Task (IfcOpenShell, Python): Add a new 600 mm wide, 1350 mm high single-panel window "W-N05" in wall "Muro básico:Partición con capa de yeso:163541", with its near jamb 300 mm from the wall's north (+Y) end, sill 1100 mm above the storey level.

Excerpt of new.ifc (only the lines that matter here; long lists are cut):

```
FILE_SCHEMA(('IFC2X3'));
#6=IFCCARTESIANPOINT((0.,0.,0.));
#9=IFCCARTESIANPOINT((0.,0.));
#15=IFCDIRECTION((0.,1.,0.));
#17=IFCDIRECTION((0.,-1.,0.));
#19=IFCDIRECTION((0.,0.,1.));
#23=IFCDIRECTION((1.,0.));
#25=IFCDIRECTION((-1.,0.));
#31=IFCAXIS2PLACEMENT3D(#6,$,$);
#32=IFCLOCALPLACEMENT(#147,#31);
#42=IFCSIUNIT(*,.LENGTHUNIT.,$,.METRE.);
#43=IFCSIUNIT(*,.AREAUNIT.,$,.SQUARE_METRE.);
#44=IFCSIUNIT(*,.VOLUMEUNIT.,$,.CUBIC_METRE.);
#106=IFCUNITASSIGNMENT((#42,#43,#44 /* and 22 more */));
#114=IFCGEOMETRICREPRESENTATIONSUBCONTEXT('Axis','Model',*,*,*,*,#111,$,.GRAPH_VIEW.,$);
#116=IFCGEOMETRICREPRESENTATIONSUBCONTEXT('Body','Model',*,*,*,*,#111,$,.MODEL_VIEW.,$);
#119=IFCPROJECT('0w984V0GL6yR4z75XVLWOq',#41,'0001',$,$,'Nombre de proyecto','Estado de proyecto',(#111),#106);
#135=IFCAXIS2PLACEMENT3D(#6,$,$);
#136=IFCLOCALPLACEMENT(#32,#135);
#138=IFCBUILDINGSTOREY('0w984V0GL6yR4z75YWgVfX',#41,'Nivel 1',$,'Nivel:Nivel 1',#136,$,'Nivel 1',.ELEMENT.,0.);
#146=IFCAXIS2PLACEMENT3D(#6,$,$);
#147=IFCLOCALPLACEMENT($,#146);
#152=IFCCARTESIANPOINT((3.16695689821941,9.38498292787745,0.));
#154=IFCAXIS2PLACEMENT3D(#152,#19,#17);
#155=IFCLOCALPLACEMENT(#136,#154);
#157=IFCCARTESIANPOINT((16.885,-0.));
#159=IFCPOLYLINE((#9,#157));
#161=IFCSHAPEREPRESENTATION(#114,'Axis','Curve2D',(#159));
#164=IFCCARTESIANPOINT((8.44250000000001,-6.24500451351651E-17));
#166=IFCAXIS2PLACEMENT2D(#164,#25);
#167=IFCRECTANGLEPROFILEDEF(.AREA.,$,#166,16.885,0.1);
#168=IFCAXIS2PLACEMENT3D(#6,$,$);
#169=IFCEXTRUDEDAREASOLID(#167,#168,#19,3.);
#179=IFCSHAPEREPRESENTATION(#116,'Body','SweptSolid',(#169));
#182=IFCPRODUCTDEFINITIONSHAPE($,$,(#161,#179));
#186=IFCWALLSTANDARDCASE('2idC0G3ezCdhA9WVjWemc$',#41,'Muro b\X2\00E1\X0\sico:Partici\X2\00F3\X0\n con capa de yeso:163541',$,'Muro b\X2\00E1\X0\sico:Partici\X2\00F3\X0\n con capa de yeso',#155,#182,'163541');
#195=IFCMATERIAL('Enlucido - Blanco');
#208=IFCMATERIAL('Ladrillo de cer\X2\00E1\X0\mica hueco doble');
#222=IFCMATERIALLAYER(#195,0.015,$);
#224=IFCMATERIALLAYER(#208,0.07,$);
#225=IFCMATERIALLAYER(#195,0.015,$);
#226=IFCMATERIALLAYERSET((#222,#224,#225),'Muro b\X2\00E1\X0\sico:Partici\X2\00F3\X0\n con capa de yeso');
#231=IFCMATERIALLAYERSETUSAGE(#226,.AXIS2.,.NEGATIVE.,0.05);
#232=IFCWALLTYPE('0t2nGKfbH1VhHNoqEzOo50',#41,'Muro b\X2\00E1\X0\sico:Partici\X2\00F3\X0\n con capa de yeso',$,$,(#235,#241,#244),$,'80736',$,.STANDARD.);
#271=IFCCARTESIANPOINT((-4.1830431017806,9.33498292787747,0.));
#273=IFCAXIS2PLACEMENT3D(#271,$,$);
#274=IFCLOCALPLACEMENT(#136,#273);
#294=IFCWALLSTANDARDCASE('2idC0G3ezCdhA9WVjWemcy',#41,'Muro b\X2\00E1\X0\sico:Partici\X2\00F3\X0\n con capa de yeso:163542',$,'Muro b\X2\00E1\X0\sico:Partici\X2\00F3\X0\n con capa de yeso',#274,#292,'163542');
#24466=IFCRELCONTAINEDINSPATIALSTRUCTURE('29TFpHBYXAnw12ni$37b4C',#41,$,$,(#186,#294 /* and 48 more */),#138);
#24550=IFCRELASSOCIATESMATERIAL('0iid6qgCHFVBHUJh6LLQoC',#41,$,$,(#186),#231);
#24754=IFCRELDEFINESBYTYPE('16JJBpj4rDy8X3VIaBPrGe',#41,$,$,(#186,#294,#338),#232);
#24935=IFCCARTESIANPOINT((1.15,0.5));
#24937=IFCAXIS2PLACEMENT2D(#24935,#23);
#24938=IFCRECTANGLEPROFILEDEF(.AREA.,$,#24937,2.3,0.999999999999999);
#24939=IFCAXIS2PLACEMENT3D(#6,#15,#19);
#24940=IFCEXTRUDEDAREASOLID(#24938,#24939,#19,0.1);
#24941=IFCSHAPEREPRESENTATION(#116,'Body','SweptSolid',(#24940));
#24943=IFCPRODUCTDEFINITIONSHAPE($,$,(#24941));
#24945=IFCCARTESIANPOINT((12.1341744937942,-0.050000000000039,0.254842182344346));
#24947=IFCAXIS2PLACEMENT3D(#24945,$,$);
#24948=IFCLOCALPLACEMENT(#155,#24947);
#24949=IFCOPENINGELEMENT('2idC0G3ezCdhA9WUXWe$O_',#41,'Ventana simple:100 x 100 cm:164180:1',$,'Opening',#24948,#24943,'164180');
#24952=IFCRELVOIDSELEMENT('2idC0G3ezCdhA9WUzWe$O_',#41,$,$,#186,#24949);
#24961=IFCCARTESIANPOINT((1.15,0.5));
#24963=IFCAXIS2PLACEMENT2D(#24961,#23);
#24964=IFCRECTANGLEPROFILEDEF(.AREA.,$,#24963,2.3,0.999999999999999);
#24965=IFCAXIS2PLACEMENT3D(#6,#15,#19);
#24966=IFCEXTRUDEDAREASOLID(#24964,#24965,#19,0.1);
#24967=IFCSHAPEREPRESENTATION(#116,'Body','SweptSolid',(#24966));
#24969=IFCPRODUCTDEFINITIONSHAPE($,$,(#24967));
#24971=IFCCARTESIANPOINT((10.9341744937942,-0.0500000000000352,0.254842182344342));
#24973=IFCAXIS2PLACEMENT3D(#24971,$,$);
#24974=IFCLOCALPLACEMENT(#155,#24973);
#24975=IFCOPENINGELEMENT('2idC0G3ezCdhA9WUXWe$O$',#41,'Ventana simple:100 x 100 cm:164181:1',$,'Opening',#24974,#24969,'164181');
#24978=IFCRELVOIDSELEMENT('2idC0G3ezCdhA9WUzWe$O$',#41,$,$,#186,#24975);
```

```python
import numpy as np
import ifcopenshell
import ifcopenshell.api.feature
import ifcopenshell.api.geometry
import ifcopenshell.api.root
import ifcopenshell.api.spatial
import ifcopenshell.api.type
import ifcopenshell.geom
import ifcopenshell.util.element
import ifcopenshell.util.placement
import ifcopenshell.util.representation
import ifcopenshell.util.shape
import ifcopenshell.util.unit

model = ifcopenshell.open("new.ifc")
unit_scale = ifcopenshell.util.unit.calculate_unit_scale(model)
settings = ifcopenshell.geom.settings()


def volume(element):
    """Net volume in cubic metres, openings subtracted."""
    shape = ifcopenshell.geom.create_shape(settings, element)
    return ifcopenshell.util.shape.get_volume(shape.geometry)


wall = model.by_id(186)
storey = ifcopenshell.util.element.get_container(wall, ifc_class="IfcBuildingStorey")
context = ifcopenshell.util.representation.get_context(model, "Model", "Body", "MODEL_VIEW")
before = volume(wall)

width, height, from_end, sill = 0.6, 1.35, 0.3, 1.1  # metres

# The wall runs along its own X axis, and the end named is its -X end.
wall_shape = ifcopenshell.geom.create_shape(settings, wall)
x, y, z = ifcopenshell.util.shape.get_vertices(wall_shape.geometry).T
start = x.min() + from_end
face, thickness = float(y.min()), float(y.max() - y.min())
wall_matrix = ifcopenshell.util.placement.get_local_placement(wall.ObjectPlacement)
level = ifcopenshell.util.placement.get_local_placement(storey.ObjectPlacement)[2, 3]


def in_wall(x, y):
    """Placement at x, y metres in the wall's axes, at sill height."""
    matrix = wall_matrix.copy()
    matrix[:, 3] = wall_matrix @ np.array([x / unit_scale, y / unit_scale, 0.0, 1.0])
    matrix[2, 3] = level + sill / unit_scale
    return matrix


# Opening: a box that overshoots both wall faces by 50 mm.
opening = ifcopenshell.api.root.create_entity(model, ifc_class="IfcOpeningElement")
box = ifcopenshell.api.geometry.add_wall_representation(
    model, context=context, length=width, height=height, thickness=thickness + 0.1
)
ifcopenshell.api.geometry.assign_representation(model, product=opening, representation=box)
ifcopenshell.api.geometry.edit_object_placement(model, product=opening, matrix=in_wall(start, face - 0.05), is_si=False)
ifcopenshell.api.feature.add_feature(model, feature=opening, element=wall)

window = ifcopenshell.api.root.create_entity(model, ifc_class="IfcWindow", name="W-N05")
window.OverallWidth, window.OverallHeight = width / unit_scale, height / unit_scale
body = ifcopenshell.api.geometry.add_window_representation(
    model,
    context=context,
    overall_width=window.OverallWidth,
    overall_height=window.OverallHeight,
    partition_type="SINGLE_PANEL",
)
ifcopenshell.api.geometry.assign_representation(model, product=window, representation=body)
ifcopenshell.api.spatial.assign_container(model, products=[window], relating_structure=storey)
fills = ifcopenshell.api.feature.add_filling(model, opening=opening, element=window)
fills.OwnerHistory = window.OwnerHistory  # required in IFC2X3

# IFC2X3 keeps the operation on the window style.
style = ifcopenshell.api.root.create_entity(model, ifc_class="IfcWindowStyle", name="W-N05")
style.OperationType, style.ConstructionType = "SINGLE_PANEL", "NOTDEFINED"
style.ParameterTakesPrecedence = style.Sizeable = False
ifcopenshell.api.type.assign_type(model, related_objects=[window], relating_type=style)

# Centre the window in the wall's thickness.
ifcopenshell.api.geometry.edit_object_placement(model, product=window, matrix=in_wall(start, face), is_si=False)
window_shape = ifcopenshell.geom.create_shape(settings, window)
depth = ifcopenshell.util.shape.get_vertices(window_shape.geometry)[:, 1]
offset = face + thickness / 2 - (depth.min() + depth.max()) / 2
ifcopenshell.api.geometry.edit_object_placement(model, product=window, matrix=in_wall(start, offset), is_si=False)

after = volume(wall)

print(f"wall volume {before:.3f} -> {after:.3f} m3")

model.write("new_v2.ifc")
```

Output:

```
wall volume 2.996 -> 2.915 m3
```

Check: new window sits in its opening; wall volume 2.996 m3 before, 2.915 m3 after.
